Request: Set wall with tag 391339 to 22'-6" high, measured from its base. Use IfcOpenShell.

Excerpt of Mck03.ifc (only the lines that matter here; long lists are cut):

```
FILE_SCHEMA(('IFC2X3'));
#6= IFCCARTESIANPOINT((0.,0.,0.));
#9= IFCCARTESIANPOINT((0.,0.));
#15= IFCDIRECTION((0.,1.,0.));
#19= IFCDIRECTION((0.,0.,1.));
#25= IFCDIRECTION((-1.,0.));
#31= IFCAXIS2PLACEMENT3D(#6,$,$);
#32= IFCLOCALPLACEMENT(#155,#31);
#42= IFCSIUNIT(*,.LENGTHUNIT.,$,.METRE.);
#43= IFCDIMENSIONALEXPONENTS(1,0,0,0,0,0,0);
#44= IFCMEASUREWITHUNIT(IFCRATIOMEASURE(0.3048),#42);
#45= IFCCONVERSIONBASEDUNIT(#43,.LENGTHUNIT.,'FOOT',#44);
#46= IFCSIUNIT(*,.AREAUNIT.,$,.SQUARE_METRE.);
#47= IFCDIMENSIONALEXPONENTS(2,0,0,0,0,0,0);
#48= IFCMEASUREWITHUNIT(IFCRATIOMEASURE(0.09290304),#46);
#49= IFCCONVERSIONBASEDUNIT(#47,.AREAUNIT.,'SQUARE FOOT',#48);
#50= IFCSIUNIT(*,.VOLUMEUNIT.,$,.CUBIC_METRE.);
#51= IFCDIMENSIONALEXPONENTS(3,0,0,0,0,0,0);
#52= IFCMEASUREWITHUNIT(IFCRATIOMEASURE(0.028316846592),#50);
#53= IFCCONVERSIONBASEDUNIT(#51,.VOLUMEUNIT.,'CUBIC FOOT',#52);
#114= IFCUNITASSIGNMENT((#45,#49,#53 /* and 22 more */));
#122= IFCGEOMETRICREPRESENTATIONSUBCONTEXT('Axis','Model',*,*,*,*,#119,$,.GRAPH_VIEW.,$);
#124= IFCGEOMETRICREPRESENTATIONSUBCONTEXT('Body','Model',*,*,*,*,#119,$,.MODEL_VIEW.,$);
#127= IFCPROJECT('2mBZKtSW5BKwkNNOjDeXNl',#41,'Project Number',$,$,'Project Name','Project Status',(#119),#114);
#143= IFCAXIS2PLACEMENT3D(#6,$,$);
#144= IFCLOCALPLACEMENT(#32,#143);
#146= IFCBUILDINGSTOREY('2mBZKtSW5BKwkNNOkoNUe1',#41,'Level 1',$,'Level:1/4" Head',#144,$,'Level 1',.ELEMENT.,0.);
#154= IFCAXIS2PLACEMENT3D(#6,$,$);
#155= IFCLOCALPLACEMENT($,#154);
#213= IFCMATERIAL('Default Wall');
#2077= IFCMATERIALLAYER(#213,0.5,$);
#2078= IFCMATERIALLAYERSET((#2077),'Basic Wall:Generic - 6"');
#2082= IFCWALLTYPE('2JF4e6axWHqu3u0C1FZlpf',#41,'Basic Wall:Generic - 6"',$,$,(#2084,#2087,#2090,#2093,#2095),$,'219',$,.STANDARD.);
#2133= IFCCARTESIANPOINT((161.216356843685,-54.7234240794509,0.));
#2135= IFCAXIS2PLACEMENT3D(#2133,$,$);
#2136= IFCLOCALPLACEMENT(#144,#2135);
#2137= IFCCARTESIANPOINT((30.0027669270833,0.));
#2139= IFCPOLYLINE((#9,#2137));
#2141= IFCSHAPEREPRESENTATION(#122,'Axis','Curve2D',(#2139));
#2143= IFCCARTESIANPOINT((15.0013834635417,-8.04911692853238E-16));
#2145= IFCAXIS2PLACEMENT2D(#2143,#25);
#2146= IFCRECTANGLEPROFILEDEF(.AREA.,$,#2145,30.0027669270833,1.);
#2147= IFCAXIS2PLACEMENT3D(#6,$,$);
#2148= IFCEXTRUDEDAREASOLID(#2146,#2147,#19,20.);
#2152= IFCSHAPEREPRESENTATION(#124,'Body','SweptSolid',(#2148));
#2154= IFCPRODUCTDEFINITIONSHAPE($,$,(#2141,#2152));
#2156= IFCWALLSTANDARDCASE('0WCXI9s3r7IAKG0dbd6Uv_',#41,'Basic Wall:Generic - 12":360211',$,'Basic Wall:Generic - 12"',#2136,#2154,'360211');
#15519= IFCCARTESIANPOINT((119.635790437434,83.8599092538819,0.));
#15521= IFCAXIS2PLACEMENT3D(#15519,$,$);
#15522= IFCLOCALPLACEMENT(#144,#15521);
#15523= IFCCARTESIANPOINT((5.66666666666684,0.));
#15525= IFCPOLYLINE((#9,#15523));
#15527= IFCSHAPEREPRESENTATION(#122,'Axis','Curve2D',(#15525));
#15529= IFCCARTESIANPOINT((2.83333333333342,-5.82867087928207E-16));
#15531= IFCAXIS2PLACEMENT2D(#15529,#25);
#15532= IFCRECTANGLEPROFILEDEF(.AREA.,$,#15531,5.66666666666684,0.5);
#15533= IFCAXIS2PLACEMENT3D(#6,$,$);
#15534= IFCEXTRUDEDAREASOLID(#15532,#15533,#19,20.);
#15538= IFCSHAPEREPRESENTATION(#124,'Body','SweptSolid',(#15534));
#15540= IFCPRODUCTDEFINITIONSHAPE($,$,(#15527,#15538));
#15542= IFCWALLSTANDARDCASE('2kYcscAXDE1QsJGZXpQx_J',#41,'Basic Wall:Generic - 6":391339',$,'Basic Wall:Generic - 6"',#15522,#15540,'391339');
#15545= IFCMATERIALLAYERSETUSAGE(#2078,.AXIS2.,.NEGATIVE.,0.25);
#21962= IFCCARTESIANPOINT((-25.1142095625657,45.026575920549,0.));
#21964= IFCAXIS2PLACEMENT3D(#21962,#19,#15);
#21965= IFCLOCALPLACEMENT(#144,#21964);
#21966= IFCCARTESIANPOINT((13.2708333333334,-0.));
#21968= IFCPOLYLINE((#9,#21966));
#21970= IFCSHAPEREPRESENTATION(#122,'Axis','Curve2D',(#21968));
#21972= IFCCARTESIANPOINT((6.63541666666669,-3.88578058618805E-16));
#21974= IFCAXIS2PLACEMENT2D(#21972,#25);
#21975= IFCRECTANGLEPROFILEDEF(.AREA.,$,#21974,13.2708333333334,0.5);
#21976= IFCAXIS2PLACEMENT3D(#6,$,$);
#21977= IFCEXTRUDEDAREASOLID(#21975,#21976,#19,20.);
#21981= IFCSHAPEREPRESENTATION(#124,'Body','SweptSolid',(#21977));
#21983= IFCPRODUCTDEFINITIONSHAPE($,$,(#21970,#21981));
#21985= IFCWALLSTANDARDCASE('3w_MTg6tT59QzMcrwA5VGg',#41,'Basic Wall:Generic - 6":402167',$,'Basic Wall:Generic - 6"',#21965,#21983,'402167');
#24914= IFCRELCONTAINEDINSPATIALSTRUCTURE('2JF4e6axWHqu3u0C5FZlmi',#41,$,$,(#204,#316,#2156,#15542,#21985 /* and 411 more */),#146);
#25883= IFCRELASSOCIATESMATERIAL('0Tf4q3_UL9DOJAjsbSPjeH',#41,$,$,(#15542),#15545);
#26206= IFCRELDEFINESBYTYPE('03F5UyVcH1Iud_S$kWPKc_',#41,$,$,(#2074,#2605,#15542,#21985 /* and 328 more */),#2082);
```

```python
import ifcopenshell
import ifcopenshell.geom
import ifcopenshell.util.representation
import ifcopenshell.util.shape
import ifcopenshell.util.unit

model = ifcopenshell.open("Mck03.ifc")
unit_scale = ifcopenshell.util.unit.calculate_unit_scale(model)
settings = ifcopenshell.geom.settings()


def volume(element):
    """Net volume in cubic metres, openings subtracted."""
    shape = ifcopenshell.geom.create_shape(settings, element)
    return ifcopenshell.util.shape.get_volume(shape.geometry)


wall = model.by_id(15542)
before = volume(wall)

body = ifcopenshell.util.representation.get_representation(wall, "Model", "Body")
solid = body.Items[0]
old_height = solid.Depth
solid.Depth = 270 * 0.0254 / unit_scale
after = volume(wall)

print(f"height {old_height:g} -> {solid.Depth:g}, volume {before:.3f} -> {after:.3f} m3")

model.write("Mck03_v2.ifc")
```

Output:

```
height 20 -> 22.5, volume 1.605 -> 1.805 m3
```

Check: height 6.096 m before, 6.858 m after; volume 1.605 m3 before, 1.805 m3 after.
